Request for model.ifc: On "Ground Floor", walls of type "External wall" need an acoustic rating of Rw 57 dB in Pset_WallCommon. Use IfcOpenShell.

First a look at what the model holds.

```python
import ifcopenshell
import ifcopenshell.util.element

model = ifcopenshell.open("model.ifc")
print(model.schema)
storey = next(s for s in model.by_type("IfcBuildingStorey") if s.Name == "Ground Floor")
walls = [e for e in ifcopenshell.util.element.get_decomposition(storey) if e.is_a("IfcWall")]
seen = {}
for e in walls:
    element_type = ifcopenshell.util.element.get_type(e)
    key = (element_type.Name if element_type != e and element_type else None, ifcopenshell.util.element.get_pset(e, "Pset_WallCommon", "AcousticRating"))
    seen[key] = seen.get(key, 0) + 1
for (name, value), count in sorted(seen.items(), key=str):
    print(count, "x", name, "|", value)
```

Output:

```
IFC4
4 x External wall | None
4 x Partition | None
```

```python
import ifcopenshell
import ifcopenshell.api.pset
import ifcopenshell.util.element

model = ifcopenshell.open("model.ifc")

storey = next(s for s in model.by_type("IfcBuildingStorey") if s.Name == "Ground Floor")
walls = [e for e in ifcopenshell.util.element.get_decomposition(storey) if e.is_a("IfcWall")]

count = 0
for e in walls:
    element_type = ifcopenshell.util.element.get_type(e)
    if element_type in (None, e) or element_type.Name != "External wall":
        continue
    # add_pset returns the element's existing set when there is one.
    pset = ifcopenshell.api.pset.add_pset(model, product=e, name="Pset_WallCommon")
    ifcopenshell.api.pset.edit_pset(model, pset=pset, properties={"AcousticRating": "Rw 57 dB"})
    count += 1

print(count, "walls updated")

model.write("model_rev.ifc")
```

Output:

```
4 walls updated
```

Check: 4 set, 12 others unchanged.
